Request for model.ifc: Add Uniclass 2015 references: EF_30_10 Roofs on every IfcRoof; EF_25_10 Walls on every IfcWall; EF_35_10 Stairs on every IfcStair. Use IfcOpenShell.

First a look at what the model holds.

```python
import ifcopenshell

model = ifcopenshell.open("model.ifc")
print(model.schema)
print("classifications:", [c.Name for c in model.by_type("IfcClassification")])
for ifc_class in ("IfcDoor", "IfcRoof", "IfcStair", "IfcWall", "IfcWindow"):
    print(ifc_class, len(model.by_type(ifc_class)))
```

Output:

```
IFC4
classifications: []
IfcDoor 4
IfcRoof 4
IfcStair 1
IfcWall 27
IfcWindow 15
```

```python
import ifcopenshell
import ifcopenshell.api.classification

model = ifcopenshell.open("model.ifc")

system = ifcopenshell.api.classification.add_classification(model, classification="Uniclass 2015")

codes = {
    "IfcRoof": ("EF_30_10", "Roofs"),
    "IfcWall": ("EF_25_10", "Walls"),
    "IfcStair": ("EF_35_10", "Stairs"),
}
for ifc_class, (code, name) in codes.items():
    products = model.by_type(ifc_class)
    ifcopenshell.api.classification.add_reference(
        model, products=products, classification=system, identification=code, name=name
    )
    print(code, len(products))

model.write("model_rev.ifc")
```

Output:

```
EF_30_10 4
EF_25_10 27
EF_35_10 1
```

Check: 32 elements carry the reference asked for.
